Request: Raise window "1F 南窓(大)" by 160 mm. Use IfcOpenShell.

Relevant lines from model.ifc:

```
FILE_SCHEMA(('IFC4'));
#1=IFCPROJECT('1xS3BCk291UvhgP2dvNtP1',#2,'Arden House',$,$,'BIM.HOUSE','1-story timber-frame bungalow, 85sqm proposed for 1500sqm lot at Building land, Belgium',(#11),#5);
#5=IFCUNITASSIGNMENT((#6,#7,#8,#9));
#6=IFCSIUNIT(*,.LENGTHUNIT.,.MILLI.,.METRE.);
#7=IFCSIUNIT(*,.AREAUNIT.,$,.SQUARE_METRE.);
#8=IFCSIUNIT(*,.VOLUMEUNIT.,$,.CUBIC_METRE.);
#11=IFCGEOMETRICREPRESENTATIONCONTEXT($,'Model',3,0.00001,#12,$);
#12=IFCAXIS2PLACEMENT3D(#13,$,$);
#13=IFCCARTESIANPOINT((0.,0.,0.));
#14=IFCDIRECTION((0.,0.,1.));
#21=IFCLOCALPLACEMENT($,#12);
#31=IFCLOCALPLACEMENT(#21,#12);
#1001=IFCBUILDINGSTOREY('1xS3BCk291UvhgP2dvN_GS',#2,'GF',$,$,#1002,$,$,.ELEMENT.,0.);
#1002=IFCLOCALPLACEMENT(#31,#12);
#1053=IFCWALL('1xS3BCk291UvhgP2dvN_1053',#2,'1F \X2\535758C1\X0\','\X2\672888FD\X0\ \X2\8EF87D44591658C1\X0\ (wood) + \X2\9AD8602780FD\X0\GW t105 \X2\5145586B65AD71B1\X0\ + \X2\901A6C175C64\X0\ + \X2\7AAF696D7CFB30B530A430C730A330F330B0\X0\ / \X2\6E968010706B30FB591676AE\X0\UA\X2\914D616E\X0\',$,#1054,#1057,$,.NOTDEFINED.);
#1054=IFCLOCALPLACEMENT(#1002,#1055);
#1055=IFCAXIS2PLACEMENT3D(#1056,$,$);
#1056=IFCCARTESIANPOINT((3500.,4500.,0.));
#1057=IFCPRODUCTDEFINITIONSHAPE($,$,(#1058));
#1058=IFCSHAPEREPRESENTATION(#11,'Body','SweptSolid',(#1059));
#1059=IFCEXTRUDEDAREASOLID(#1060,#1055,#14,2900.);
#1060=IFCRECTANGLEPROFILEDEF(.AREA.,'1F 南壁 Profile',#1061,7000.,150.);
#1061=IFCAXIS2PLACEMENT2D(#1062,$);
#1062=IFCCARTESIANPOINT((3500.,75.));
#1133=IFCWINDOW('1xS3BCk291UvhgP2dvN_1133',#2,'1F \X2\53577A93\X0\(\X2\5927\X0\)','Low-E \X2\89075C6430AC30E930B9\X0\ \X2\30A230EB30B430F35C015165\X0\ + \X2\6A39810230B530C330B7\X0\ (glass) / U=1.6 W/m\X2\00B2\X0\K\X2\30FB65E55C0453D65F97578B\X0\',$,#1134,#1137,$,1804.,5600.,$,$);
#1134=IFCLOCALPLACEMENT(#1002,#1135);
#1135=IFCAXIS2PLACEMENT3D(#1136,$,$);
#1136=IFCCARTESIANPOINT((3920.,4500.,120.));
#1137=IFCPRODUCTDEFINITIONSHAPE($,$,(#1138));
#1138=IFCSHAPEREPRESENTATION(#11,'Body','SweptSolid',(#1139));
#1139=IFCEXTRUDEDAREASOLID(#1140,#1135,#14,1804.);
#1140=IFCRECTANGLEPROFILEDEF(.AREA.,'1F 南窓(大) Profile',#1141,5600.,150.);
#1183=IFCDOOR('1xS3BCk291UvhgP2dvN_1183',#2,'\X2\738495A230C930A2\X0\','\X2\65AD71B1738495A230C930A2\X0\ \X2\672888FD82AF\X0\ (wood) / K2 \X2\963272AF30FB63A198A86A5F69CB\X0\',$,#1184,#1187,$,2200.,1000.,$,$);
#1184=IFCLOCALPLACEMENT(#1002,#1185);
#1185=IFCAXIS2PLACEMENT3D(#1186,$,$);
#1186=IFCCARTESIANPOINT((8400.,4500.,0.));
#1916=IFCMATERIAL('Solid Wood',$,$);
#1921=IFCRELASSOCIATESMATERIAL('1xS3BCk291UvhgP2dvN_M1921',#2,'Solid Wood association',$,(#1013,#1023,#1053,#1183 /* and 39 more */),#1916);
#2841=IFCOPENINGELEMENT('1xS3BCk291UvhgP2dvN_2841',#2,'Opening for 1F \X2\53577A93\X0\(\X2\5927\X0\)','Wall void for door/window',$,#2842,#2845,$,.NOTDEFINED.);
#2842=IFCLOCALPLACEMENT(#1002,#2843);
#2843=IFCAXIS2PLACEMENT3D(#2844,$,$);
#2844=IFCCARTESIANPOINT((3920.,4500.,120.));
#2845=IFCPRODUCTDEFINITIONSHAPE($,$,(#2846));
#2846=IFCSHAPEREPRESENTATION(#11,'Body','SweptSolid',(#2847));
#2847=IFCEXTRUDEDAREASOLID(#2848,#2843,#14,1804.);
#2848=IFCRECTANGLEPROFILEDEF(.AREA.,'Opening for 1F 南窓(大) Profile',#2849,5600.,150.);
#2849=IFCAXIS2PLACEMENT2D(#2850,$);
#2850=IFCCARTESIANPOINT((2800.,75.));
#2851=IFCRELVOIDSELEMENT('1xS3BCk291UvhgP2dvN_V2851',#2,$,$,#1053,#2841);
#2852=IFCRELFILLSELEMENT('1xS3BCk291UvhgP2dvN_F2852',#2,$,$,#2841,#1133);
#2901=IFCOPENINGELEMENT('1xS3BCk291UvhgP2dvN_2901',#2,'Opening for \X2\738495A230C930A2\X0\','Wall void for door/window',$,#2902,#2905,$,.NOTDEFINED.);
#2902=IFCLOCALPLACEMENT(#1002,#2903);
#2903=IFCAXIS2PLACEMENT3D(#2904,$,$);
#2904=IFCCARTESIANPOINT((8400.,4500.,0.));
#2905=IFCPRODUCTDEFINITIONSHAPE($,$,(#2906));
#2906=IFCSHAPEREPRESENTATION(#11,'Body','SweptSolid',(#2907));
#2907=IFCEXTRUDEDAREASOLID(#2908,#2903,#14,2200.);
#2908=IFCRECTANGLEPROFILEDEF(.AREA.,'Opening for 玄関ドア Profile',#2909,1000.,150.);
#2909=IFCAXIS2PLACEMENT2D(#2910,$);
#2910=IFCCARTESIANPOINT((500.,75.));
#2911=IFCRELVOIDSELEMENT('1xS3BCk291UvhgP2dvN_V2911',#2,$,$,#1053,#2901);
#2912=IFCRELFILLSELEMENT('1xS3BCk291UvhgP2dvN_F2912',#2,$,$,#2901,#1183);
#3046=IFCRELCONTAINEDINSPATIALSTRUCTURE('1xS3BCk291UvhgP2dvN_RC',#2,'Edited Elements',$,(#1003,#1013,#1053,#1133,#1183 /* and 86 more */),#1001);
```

```python
import numpy as np
import ifcopenshell
import ifcopenshell.api.geometry
import ifcopenshell.util.placement
import ifcopenshell.util.unit

model = ifcopenshell.open("model.ifc")
unit_scale = ifcopenshell.util.unit.calculate_unit_scale(model)

window = model.by_guid("1xS3BCk291UvhgP2dvN_1133")
opening = window.FillsVoids[0].RelatingOpeningElement
dz = 160.0

shift = np.array([0.0, 0.0, dz])
# The window is not placed relative to its opening, so move both.
for product in (opening, window):
    matrix = ifcopenshell.util.placement.get_local_placement(product.ObjectPlacement)
    matrix[:3, 3] += shift
    ifcopenshell.api.geometry.edit_object_placement(model, product=product, matrix=matrix, is_si=False)

print(f"moved by {dz * unit_scale:+.3f} m")

model.write("model-out.ifc")
```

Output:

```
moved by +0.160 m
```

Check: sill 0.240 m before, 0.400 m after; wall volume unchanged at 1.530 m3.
